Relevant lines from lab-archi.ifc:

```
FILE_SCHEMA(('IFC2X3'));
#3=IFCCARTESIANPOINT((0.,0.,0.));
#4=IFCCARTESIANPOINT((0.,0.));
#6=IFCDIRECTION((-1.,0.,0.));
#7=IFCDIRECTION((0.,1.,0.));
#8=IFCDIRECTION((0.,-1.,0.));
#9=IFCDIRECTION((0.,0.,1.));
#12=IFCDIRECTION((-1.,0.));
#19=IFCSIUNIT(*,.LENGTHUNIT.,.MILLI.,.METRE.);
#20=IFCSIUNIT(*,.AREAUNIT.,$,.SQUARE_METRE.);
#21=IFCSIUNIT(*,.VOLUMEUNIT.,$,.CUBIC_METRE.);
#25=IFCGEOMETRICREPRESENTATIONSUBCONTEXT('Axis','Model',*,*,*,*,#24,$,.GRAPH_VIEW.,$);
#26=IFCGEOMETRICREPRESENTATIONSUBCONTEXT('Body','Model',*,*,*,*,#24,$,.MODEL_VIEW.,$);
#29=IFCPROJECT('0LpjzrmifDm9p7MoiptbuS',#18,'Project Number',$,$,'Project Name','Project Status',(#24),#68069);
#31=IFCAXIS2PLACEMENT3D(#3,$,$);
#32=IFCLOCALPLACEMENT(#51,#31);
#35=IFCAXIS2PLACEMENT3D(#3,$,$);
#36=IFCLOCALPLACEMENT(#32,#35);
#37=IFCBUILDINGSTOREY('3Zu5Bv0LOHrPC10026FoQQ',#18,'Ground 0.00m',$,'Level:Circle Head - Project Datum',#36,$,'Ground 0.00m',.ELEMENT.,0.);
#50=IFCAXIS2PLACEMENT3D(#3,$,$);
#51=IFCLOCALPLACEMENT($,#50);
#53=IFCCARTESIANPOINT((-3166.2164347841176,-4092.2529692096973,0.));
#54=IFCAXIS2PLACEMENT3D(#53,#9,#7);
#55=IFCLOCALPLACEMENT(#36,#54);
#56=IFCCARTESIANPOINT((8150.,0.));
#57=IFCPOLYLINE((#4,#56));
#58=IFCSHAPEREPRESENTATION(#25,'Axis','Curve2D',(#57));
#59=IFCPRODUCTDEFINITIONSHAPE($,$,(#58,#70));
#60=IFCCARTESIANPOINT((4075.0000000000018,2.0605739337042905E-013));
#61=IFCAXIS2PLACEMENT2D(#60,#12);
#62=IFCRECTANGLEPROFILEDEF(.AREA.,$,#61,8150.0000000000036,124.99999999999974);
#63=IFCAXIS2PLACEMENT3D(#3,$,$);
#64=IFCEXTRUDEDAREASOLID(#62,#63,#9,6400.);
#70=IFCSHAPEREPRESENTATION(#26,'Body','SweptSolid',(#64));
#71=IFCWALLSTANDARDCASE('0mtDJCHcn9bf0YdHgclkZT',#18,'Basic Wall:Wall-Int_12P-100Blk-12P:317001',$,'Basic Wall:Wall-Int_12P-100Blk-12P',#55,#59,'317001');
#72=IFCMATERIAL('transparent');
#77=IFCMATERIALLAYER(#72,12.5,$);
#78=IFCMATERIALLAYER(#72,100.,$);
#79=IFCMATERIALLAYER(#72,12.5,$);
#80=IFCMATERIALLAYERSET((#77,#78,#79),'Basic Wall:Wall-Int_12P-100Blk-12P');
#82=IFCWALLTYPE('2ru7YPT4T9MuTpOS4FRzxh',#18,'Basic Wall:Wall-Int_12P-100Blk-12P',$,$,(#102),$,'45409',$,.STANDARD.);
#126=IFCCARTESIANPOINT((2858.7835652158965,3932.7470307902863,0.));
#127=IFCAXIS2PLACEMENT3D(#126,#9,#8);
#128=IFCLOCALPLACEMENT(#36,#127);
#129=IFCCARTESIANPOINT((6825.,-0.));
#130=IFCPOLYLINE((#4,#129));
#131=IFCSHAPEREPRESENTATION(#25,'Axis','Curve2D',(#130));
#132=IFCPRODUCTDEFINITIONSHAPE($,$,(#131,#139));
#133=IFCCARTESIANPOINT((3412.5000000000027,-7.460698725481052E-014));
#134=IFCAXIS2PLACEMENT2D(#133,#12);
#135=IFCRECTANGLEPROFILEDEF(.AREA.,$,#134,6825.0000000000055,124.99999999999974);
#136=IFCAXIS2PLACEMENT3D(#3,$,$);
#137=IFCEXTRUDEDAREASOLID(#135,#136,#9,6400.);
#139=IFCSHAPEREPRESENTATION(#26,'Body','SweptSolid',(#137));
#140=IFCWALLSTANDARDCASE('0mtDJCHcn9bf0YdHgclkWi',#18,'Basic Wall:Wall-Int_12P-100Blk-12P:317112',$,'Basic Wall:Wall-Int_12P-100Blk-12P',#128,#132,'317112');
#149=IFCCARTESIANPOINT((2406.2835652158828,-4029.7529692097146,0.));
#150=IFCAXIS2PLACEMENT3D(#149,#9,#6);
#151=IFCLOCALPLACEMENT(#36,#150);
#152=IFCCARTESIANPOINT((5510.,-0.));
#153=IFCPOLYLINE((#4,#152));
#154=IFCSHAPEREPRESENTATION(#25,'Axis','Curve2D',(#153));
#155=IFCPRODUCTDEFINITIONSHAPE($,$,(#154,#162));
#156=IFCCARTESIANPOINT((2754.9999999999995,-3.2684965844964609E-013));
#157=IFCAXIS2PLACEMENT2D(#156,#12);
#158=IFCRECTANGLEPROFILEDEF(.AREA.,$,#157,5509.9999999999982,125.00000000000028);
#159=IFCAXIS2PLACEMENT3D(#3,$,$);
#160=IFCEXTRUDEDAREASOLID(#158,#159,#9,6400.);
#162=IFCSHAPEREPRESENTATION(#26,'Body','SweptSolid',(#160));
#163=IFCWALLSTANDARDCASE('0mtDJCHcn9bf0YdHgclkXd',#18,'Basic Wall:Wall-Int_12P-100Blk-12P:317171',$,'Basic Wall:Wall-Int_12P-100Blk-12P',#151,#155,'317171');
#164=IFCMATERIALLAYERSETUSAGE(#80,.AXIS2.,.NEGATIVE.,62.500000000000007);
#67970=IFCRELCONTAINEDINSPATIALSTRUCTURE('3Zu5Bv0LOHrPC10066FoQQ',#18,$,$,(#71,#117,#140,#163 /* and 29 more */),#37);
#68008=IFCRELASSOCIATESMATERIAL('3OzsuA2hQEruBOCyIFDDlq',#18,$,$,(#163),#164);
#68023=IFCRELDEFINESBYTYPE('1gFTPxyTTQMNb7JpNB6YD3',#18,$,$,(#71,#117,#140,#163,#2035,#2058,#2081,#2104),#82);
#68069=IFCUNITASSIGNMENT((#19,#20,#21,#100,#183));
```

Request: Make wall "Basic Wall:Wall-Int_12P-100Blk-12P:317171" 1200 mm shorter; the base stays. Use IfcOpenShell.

```python
import ifcopenshell
import ifcopenshell.geom
import ifcopenshell.util.representation
import ifcopenshell.util.shape
import ifcopenshell.util.unit

model = ifcopenshell.open("lab-archi.ifc")
unit_scale = ifcopenshell.util.unit.calculate_unit_scale(model)
settings = ifcopenshell.geom.settings()


def volume(element):
    """Net volume in cubic metres, openings subtracted."""
    shape = ifcopenshell.geom.create_shape(settings, element)
    return ifcopenshell.util.shape.get_volume(shape.geometry)


wall = model.by_id(163)
before = volume(wall)

body = ifcopenshell.util.representation.get_representation(wall, "Model", "Body")
solid = body.Items[0]
old_height = solid.Depth
solid.Depth -= 1.2 / unit_scale
after = volume(wall)

print(f"height {old_height:g} -> {solid.Depth:g}, volume {before:.3f} -> {after:.3f} m3")

model.write("lab-archi_rev.ifc")
```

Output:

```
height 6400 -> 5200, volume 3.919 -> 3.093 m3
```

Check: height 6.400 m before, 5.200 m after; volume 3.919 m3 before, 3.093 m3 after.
